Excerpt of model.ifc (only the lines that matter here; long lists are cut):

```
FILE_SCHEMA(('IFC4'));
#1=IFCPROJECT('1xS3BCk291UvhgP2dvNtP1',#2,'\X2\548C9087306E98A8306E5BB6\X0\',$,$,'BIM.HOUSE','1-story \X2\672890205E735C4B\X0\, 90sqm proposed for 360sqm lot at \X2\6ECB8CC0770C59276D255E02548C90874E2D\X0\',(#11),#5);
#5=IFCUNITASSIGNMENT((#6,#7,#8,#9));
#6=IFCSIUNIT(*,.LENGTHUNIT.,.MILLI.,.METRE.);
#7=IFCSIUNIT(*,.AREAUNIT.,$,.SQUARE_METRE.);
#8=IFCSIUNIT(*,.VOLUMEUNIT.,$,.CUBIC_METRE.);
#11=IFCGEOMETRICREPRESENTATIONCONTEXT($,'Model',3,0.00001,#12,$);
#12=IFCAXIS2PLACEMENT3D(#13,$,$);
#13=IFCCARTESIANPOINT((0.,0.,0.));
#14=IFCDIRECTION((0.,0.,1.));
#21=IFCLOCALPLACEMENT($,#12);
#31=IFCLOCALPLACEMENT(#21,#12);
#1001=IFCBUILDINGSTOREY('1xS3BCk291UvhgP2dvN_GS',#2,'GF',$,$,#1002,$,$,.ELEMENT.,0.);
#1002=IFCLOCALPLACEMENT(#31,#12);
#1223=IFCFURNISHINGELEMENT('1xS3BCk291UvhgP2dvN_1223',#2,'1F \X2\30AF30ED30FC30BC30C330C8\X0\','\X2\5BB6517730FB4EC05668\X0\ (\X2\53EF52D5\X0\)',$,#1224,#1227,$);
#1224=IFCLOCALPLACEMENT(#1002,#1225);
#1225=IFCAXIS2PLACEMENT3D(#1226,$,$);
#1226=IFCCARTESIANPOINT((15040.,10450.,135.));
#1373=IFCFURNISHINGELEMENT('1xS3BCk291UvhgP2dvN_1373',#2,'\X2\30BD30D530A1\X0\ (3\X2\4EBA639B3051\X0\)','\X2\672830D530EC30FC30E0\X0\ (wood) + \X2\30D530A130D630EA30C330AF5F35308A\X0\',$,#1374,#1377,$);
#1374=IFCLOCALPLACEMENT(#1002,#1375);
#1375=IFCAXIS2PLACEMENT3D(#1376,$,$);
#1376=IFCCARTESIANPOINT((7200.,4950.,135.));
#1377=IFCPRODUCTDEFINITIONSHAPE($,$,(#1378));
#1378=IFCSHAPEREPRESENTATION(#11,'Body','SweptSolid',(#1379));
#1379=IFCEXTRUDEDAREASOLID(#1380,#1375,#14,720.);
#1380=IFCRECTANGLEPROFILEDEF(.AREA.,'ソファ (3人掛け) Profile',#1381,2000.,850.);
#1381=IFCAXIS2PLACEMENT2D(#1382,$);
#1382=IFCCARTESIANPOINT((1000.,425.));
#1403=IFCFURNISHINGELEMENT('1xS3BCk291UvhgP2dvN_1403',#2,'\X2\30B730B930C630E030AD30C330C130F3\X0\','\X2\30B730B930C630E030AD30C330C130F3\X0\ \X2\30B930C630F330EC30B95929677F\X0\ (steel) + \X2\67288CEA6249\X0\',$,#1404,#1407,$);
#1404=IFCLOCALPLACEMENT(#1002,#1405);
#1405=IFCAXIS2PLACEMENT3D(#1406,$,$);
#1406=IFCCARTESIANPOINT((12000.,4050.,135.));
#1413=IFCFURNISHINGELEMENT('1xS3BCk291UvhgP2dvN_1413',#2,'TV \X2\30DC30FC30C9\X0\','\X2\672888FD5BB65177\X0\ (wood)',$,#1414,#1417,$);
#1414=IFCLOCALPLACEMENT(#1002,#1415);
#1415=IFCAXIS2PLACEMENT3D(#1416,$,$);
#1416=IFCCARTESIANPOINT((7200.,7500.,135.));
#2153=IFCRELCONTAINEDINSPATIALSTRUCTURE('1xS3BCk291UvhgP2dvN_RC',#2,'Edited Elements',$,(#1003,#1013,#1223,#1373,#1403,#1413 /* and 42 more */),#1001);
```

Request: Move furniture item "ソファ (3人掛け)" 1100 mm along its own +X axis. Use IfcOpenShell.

```python
import ifcopenshell
import ifcopenshell.api.geometry
import ifcopenshell.util.placement
import ifcopenshell.util.unit

model = ifcopenshell.open("model.ifc")
unit_scale = ifcopenshell.util.unit.calculate_unit_scale(model)

item = model.by_guid("1xS3BCk291UvhgP2dvN_1373")
matrix = ifcopenshell.util.placement.get_local_placement(item.ObjectPlacement)
matrix[:3, 3] += matrix[:3, 0] * 1.1 / unit_scale
ifcopenshell.api.geometry.edit_object_placement(model, product=item, matrix=matrix, is_si=False)

print(ifcopenshell.util.placement.get_local_placement(item.ObjectPlacement).round(3) + 0.0)

model.write("model_rev.ifc")
```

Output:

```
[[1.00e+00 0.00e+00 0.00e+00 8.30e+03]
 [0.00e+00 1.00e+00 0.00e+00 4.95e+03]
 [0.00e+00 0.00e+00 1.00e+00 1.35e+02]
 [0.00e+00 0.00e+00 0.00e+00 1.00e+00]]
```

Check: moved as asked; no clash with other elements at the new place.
